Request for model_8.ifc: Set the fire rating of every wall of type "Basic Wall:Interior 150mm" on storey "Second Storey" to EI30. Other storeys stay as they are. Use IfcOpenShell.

First a look at what the model holds.

```python
import ifcopenshell
import ifcopenshell.util.element

model = ifcopenshell.open("model_8.ifc")
print(model.schema)
storey = next(s for s in model.by_type("IfcBuildingStorey") if s.Name == "Second Storey")
walls = [e for e in ifcopenshell.util.element.get_decomposition(storey) if e.is_a("IfcWall")]
seen = {}
for e in walls:
    element_type = ifcopenshell.util.element.get_type(e)
    key = (element_type.Name if element_type != e and element_type else None, ifcopenshell.util.element.get_pset(e, "Pset_WallCommon", "FireRating"))
    seen[key] = seen.get(key, 0) + 1
for (name, value), count in sorted(seen.items(), key=str):
    print(count, "x", name, "|", value)
```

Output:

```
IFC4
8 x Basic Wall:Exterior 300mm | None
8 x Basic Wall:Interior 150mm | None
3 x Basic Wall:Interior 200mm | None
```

```python
import ifcopenshell
import ifcopenshell.api.pset
import ifcopenshell.util.element

model = ifcopenshell.open("model_8.ifc")

storey = next(s for s in model.by_type("IfcBuildingStorey") if s.Name == "Second Storey")
walls = [e for e in ifcopenshell.util.element.get_decomposition(storey) if e.is_a("IfcWall")]

count = 0
for e in walls:
    element_type = ifcopenshell.util.element.get_type(e)
    if element_type in (None, e) or element_type.Name != "Basic Wall:Interior 150mm":
        continue
    # add_pset returns the element's existing set when there is one.
    pset = ifcopenshell.api.pset.add_pset(model, product=e, name="Pset_WallCommon")
    ifcopenshell.api.pset.edit_pset(model, pset=pset, properties={"FireRating": "EI30"})
    count += 1

print(count, "walls updated")

model.write("model_8_edited.ifc")
```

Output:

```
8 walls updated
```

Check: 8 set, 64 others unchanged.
